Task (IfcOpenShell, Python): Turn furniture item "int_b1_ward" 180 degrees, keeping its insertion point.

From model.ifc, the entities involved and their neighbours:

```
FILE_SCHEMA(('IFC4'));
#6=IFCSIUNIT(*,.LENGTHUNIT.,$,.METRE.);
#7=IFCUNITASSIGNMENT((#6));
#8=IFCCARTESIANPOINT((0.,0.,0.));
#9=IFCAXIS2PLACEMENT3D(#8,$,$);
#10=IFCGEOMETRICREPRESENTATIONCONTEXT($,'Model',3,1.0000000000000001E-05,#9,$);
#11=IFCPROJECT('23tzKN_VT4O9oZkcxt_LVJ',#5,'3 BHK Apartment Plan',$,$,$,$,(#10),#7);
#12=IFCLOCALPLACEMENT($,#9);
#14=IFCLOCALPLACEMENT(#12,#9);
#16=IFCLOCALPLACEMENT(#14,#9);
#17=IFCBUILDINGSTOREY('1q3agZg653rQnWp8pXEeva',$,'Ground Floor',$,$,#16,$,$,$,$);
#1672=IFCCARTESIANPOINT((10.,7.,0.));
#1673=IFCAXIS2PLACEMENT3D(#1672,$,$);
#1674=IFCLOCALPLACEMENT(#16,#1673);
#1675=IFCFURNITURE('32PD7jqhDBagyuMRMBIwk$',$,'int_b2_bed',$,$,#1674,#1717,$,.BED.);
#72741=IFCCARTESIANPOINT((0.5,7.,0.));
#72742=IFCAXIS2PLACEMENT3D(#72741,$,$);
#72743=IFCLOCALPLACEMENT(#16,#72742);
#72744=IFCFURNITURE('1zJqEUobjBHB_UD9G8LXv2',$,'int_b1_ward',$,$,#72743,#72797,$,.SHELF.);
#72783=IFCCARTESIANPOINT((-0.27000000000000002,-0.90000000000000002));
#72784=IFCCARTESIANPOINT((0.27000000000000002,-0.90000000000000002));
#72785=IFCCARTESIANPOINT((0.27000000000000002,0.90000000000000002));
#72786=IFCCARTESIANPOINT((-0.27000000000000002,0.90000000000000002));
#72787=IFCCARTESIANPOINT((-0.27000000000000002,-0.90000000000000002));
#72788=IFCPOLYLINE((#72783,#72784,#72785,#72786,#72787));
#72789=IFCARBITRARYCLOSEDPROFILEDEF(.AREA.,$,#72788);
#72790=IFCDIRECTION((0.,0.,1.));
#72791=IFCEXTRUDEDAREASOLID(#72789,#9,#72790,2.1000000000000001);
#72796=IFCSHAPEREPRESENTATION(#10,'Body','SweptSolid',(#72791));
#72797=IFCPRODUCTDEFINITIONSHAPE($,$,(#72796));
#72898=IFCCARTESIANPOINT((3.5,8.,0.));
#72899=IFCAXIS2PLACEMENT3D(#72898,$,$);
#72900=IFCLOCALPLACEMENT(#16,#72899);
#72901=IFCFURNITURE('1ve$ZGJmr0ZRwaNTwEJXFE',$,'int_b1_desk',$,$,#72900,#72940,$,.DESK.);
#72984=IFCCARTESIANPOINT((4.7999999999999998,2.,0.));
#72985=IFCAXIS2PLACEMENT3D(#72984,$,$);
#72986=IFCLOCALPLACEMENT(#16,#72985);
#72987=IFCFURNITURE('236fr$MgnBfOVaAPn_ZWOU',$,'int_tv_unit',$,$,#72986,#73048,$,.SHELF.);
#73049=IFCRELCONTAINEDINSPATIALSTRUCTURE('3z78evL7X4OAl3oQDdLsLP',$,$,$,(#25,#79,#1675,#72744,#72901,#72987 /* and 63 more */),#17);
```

```python
import ifcopenshell
import ifcopenshell.api.geometry
import ifcopenshell.util.placement

model = ifcopenshell.open("model.ifc")

item = model.by_guid("1zJqEUobjBHB_UD9G8LXv2")
matrix = ifcopenshell.util.placement.get_local_placement(item.ObjectPlacement)
matrix = matrix @ ifcopenshell.util.placement.rotation(180, "Z")
ifcopenshell.api.geometry.edit_object_placement(model, product=item, matrix=matrix, is_si=False)

print(ifcopenshell.util.placement.get_local_placement(item.ObjectPlacement).round(3) + 0.0)

model.write("model_v2.ifc")
```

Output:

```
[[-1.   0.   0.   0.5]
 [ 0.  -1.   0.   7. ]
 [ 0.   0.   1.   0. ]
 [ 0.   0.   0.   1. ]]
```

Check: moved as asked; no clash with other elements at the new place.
